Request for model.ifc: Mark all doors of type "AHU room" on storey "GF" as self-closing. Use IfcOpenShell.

First a look at what the model holds.

```python
import ifcopenshell
import ifcopenshell.util.element

model = ifcopenshell.open("model.ifc")
print(model.schema)
storey = next(s for s in model.by_type("IfcBuildingStorey") if s.Name == "GF")
doors = [e for e in ifcopenshell.util.element.get_decomposition(storey) if e.is_a("IfcDoor")]
seen = {}
for e in doors:
    element_type = ifcopenshell.util.element.get_type(e)
    key = (element_type.Name if element_type != e and element_type else None, ifcopenshell.util.element.get_pset(e, "Pset_DoorCommon", "SelfClosing"))
    seen[key] = seen.get(key, 0) + 1
for (name, value), count in sorted(seen.items(), key=str):
    print(count, "x", name, "|", value)
```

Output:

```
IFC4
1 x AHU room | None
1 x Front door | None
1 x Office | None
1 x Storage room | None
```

```python
import ifcopenshell
import ifcopenshell.api.pset
import ifcopenshell.util.element

model = ifcopenshell.open("model.ifc")

storey = next(s for s in model.by_type("IfcBuildingStorey") if s.Name == "GF")
doors = [e for e in ifcopenshell.util.element.get_decomposition(storey) if e.is_a("IfcDoor")]

count = 0
for e in doors:
    element_type = ifcopenshell.util.element.get_type(e)
    if element_type in (None, e) or element_type.Name != "AHU room":
        continue
    # add_pset returns the element's existing set when there is one.
    pset = ifcopenshell.api.pset.add_pset(model, product=e, name="Pset_DoorCommon")
    ifcopenshell.api.pset.edit_pset(model, pset=pset, properties={"SelfClosing": True})
    count += 1

print(count, "doors updated")

model.write("model_v2.ifc")
```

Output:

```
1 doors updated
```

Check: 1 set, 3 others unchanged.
